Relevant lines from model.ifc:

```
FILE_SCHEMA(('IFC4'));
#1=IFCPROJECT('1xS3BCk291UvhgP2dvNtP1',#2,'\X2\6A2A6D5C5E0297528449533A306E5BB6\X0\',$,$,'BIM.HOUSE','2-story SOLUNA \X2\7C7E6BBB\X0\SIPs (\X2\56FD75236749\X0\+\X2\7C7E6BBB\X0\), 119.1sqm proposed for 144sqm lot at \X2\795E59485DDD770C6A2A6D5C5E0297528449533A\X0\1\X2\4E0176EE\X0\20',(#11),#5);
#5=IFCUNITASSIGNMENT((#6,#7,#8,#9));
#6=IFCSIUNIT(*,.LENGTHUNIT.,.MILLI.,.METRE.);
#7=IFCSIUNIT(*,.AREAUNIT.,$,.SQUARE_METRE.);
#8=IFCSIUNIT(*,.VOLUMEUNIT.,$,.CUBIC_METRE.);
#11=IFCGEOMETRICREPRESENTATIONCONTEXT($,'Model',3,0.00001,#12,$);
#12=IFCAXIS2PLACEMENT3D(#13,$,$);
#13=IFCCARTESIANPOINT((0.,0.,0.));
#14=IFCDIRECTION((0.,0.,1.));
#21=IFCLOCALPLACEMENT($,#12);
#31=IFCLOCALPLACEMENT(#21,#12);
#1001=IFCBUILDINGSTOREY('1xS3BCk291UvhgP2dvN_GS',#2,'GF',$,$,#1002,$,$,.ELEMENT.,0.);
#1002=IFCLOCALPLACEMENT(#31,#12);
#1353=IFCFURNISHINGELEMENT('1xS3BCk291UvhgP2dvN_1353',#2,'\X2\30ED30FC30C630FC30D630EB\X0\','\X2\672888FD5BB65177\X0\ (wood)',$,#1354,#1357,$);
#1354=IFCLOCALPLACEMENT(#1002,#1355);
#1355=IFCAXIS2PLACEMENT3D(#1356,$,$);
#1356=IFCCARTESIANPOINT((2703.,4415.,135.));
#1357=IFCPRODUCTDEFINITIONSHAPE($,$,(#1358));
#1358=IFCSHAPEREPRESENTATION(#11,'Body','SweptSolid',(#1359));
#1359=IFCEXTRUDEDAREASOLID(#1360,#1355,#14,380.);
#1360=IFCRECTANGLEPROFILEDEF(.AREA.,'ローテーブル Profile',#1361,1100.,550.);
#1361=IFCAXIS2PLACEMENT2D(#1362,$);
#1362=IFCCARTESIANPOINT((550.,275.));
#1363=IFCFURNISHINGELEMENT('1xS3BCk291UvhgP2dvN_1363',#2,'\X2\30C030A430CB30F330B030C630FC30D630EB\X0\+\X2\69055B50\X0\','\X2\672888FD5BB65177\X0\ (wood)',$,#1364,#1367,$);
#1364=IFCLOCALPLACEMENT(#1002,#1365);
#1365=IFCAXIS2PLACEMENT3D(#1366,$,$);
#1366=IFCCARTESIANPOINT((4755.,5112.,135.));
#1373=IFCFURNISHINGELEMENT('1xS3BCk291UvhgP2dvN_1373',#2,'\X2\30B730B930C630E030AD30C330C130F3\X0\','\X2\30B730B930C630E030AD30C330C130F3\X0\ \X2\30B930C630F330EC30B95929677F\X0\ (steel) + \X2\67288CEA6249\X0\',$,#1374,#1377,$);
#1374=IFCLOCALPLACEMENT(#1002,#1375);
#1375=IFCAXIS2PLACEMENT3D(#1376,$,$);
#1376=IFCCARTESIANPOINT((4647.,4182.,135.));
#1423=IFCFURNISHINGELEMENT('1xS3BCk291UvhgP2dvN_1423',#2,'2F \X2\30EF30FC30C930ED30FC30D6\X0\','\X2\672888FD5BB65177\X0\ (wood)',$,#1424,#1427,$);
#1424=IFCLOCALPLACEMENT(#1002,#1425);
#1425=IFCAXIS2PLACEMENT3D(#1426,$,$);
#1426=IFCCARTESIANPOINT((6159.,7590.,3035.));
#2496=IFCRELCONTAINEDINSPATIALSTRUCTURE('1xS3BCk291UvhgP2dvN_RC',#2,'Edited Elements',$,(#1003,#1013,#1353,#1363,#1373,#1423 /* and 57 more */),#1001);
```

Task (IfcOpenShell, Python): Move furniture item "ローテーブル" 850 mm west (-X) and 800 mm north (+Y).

```python
import ifcopenshell
import ifcopenshell.api.geometry
import ifcopenshell.util.placement
import ifcopenshell.util.unit

model = ifcopenshell.open("model.ifc")
unit_scale = ifcopenshell.util.unit.calculate_unit_scale(model)

item = model.by_guid("1xS3BCk291UvhgP2dvN_1353")
matrix = ifcopenshell.util.placement.get_local_placement(item.ObjectPlacement)
matrix[0, 3] -= 0.85 / unit_scale
matrix[1, 3] += 0.8 / unit_scale
ifcopenshell.api.geometry.edit_object_placement(model, product=item, matrix=matrix, is_si=False)

print(ifcopenshell.util.placement.get_local_placement(item.ObjectPlacement).round(3) + 0.0)

model.write("model_rev.ifc")
```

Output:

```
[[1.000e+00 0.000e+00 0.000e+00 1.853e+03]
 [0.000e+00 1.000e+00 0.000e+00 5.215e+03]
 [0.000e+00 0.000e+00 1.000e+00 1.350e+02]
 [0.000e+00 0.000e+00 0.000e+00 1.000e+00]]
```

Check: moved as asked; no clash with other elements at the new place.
